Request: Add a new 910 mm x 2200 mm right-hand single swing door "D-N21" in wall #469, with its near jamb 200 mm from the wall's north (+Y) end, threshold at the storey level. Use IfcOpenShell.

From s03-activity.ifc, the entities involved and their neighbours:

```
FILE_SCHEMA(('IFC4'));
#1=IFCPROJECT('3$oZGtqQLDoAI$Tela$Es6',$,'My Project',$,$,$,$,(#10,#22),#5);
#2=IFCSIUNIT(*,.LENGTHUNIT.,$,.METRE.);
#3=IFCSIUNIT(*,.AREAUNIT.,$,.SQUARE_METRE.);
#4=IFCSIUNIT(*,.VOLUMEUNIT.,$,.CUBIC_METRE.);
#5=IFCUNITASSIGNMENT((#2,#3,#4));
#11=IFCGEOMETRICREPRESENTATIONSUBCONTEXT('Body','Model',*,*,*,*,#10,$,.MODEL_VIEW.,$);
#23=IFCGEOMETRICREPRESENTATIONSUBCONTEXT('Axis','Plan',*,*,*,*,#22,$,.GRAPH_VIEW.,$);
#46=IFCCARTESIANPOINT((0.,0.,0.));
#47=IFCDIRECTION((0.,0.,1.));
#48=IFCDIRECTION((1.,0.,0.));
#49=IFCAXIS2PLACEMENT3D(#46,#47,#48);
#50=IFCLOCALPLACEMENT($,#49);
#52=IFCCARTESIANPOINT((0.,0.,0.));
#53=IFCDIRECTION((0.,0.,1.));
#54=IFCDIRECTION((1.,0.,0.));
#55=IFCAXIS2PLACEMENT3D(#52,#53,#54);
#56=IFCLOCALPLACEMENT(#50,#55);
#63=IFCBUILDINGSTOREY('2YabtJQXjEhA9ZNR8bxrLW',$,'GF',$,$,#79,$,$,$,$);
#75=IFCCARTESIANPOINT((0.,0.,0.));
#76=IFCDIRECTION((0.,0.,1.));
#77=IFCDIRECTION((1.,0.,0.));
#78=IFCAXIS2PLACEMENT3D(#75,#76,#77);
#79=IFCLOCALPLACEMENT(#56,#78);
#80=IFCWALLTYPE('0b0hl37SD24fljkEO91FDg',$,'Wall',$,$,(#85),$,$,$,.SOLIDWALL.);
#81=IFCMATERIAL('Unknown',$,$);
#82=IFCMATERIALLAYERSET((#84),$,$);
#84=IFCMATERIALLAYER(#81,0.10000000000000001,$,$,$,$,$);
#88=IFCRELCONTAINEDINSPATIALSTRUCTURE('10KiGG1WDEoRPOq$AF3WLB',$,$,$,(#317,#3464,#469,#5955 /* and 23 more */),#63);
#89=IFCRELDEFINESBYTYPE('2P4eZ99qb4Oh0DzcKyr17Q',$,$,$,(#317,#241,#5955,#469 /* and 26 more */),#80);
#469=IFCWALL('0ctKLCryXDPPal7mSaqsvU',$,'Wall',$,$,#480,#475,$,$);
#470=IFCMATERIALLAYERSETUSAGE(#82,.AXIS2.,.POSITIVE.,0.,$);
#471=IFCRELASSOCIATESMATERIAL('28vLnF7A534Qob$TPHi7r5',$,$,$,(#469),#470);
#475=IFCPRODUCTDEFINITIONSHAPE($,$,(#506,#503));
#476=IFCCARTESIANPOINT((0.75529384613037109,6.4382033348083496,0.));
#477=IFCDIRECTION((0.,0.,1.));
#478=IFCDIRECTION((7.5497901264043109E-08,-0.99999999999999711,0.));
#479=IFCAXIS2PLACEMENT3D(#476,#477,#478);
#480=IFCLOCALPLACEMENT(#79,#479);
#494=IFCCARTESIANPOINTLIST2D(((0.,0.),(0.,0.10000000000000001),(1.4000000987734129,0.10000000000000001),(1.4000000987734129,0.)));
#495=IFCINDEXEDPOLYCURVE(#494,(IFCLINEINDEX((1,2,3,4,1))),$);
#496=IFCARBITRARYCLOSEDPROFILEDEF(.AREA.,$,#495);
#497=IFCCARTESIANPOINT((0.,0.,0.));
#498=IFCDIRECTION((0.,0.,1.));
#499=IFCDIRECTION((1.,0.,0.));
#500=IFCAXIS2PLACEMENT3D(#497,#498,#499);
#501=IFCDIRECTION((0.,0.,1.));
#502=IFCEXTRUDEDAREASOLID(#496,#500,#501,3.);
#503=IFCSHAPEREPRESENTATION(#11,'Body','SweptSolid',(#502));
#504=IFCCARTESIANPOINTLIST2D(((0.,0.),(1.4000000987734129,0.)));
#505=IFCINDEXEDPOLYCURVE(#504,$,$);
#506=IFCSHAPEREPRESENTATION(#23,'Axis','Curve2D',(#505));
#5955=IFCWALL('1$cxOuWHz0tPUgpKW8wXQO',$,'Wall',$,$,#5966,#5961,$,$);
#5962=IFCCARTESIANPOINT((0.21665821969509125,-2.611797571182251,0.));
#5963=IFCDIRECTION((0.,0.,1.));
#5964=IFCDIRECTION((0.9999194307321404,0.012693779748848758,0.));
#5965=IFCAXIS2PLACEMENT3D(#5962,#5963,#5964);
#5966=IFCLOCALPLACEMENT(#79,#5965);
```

```python
import numpy as np
import ifcopenshell
import ifcopenshell.api.feature
import ifcopenshell.api.geometry
import ifcopenshell.api.root
import ifcopenshell.api.spatial
import ifcopenshell.geom
import ifcopenshell.util.element
import ifcopenshell.util.placement
import ifcopenshell.util.representation
import ifcopenshell.util.shape
import ifcopenshell.util.unit

model = ifcopenshell.open("s03-activity.ifc")
unit_scale = ifcopenshell.util.unit.calculate_unit_scale(model)
settings = ifcopenshell.geom.settings()


def volume(element):
    """Net volume in cubic metres, openings subtracted."""
    shape = ifcopenshell.geom.create_shape(settings, element)
    return ifcopenshell.util.shape.get_volume(shape.geometry)


wall = model.by_guid("0ctKLCryXDPPal7mSaqsvU")
storey = ifcopenshell.util.element.get_container(wall, ifc_class="IfcBuildingStorey")
context = ifcopenshell.util.representation.get_context(model, "Model", "Body", "MODEL_VIEW")
before = volume(wall)

width, height, from_end, sill = 0.91, 2.2, 0.2, 0.0  # metres

# The wall runs along its own X axis, and the end named is its -X end.
wall_shape = ifcopenshell.geom.create_shape(settings, wall)
x, y, z = ifcopenshell.util.shape.get_vertices(wall_shape.geometry).T
start = x.min() + from_end
face, thickness = float(y.min()), float(y.max() - y.min())
wall_matrix = ifcopenshell.util.placement.get_local_placement(wall.ObjectPlacement)
level = ifcopenshell.util.placement.get_local_placement(storey.ObjectPlacement)[2, 3]


def in_wall(x, y):
    """Placement at x, y metres in the wall's axes, at sill height."""
    matrix = wall_matrix.copy()
    matrix[:, 3] = wall_matrix @ np.array([x / unit_scale, y / unit_scale, 0.0, 1.0])
    matrix[2, 3] = level + sill / unit_scale
    return matrix


# Opening: a box that overshoots both wall faces by 50 mm.
opening = ifcopenshell.api.root.create_entity(model, ifc_class="IfcOpeningElement", predefined_type="OPENING")
box = ifcopenshell.api.geometry.add_wall_representation(
    model, context=context, length=width, height=height, thickness=thickness + 0.1
)
ifcopenshell.api.geometry.assign_representation(model, product=opening, representation=box)
ifcopenshell.api.geometry.edit_object_placement(model, product=opening, matrix=in_wall(start, face - 0.05), is_si=False)
ifcopenshell.api.feature.add_feature(model, feature=opening, element=wall)

door = ifcopenshell.api.root.create_entity(model, ifc_class="IfcDoor", name="D-N21", predefined_type="DOOR")
door.OverallWidth, door.OverallHeight = width / unit_scale, height / unit_scale
door.OperationType = "SINGLE_SWING_RIGHT"
body = ifcopenshell.api.geometry.add_door_representation(
    model,
    context=context,
    overall_width=door.OverallWidth,
    overall_height=door.OverallHeight,
    operation_type="SINGLE_SWING_RIGHT",
    lining_properties={"LiningDepth": thickness / unit_scale, "ThresholdDepth": thickness / unit_scale},
)
ifcopenshell.api.geometry.assign_representation(model, product=door, representation=body)
ifcopenshell.api.spatial.assign_container(model, products=[door], relating_structure=storey)
ifcopenshell.api.feature.add_filling(model, opening=opening, element=door)

# The lining spans the wall, so the door starts at the wall face.
ifcopenshell.api.geometry.edit_object_placement(model, product=door, matrix=in_wall(start, face), is_si=False)

after = volume(wall)

print(f"wall volume {before:.3f} -> {after:.3f} m3")

model.write("s03-activity-out.ifc")
```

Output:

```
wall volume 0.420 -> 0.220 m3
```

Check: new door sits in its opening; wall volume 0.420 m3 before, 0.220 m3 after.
